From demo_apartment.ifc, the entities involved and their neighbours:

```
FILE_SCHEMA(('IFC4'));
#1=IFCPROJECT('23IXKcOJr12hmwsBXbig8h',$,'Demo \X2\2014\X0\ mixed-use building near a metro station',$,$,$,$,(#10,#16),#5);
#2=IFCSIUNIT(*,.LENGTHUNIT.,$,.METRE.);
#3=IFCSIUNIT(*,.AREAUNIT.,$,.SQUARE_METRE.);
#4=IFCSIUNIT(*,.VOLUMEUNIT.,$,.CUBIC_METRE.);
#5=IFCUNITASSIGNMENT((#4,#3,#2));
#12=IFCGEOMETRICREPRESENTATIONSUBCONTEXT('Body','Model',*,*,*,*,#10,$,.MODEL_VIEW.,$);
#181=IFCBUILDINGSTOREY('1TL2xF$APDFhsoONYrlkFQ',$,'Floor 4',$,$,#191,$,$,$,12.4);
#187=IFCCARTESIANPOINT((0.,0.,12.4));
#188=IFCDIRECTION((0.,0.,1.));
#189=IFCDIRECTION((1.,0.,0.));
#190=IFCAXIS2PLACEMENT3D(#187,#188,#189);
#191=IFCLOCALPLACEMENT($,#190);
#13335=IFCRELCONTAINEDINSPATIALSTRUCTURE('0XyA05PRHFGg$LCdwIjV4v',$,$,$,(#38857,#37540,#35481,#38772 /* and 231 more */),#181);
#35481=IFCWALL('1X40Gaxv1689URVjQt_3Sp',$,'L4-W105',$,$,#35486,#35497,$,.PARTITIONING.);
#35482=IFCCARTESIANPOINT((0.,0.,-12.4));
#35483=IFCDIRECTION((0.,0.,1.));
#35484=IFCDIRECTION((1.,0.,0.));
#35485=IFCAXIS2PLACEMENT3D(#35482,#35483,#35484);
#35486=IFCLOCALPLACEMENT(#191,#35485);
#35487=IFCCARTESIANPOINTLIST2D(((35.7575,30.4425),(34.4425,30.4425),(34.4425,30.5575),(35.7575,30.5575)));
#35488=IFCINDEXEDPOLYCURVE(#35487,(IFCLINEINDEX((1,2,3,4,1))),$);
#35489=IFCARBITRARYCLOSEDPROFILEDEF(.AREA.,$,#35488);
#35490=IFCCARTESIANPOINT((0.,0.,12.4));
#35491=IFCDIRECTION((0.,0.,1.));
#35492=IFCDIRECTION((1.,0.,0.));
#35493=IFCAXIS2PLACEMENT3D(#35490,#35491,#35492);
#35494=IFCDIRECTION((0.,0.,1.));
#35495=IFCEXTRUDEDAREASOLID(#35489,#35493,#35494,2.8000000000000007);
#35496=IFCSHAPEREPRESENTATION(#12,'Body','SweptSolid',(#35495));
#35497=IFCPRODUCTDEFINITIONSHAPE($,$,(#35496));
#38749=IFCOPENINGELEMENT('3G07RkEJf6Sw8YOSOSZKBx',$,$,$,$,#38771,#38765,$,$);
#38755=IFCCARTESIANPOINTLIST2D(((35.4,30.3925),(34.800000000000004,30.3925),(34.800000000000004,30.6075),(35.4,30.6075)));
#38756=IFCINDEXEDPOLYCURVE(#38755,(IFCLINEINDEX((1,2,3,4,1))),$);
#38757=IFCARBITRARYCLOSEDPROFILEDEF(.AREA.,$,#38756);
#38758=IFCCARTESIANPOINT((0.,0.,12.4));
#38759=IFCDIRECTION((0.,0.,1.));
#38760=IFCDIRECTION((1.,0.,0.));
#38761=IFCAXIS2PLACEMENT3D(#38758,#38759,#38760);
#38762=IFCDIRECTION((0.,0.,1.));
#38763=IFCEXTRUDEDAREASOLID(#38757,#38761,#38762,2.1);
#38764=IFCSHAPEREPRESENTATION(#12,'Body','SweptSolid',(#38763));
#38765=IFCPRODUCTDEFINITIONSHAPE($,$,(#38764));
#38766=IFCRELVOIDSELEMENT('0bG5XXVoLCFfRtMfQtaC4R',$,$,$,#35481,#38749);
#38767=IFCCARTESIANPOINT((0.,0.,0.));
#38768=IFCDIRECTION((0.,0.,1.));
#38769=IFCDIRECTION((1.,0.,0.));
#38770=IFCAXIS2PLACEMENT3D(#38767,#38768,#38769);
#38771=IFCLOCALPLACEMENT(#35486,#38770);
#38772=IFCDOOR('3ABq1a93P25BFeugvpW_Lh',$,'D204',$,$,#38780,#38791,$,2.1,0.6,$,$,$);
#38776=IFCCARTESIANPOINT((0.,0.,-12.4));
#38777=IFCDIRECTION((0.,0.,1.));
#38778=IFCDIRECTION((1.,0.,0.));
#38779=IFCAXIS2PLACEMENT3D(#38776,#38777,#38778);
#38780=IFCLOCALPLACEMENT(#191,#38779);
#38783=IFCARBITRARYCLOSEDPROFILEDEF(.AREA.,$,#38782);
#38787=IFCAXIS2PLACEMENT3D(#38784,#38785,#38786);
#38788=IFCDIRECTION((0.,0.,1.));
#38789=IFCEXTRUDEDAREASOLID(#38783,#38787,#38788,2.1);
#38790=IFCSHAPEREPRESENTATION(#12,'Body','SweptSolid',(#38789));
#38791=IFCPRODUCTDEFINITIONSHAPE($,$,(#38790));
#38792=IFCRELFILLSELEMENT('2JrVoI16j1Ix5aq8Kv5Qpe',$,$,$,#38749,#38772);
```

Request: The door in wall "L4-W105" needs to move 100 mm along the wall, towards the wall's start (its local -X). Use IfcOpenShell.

```python
import ifcopenshell
import ifcopenshell.api.geometry
import ifcopenshell.util.placement

model = ifcopenshell.open("demo_apartment.ifc")

door = model.by_guid("3ABq1a93P25BFeugvpW_Lh")
opening = door.FillsVoids[0].RelatingOpeningElement
wall = opening.VoidsElements[0].RelatingBuildingElement

wall_matrix = ifcopenshell.util.placement.get_local_placement(wall.ObjectPlacement)
shift = wall_matrix[:3, 0] * -0.1
before = ifcopenshell.util.placement.get_local_placement(door.ObjectPlacement)[:3, 3].copy()

# The door is not placed relative to its opening, so move both.
for product in (opening, door):
    matrix = ifcopenshell.util.placement.get_local_placement(product.ObjectPlacement)
    matrix[:3, 3] += shift
    ifcopenshell.api.geometry.edit_object_placement(model, product=product, matrix=matrix, is_si=False)

after = ifcopenshell.util.placement.get_local_placement(door.ObjectPlacement)[:3, 3]
print("door moved by", (after - before).round(3) + 0.0)

model.write("demo_apartment-out.ifc")
```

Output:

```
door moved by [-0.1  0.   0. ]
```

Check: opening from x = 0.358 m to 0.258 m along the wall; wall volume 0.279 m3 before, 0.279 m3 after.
